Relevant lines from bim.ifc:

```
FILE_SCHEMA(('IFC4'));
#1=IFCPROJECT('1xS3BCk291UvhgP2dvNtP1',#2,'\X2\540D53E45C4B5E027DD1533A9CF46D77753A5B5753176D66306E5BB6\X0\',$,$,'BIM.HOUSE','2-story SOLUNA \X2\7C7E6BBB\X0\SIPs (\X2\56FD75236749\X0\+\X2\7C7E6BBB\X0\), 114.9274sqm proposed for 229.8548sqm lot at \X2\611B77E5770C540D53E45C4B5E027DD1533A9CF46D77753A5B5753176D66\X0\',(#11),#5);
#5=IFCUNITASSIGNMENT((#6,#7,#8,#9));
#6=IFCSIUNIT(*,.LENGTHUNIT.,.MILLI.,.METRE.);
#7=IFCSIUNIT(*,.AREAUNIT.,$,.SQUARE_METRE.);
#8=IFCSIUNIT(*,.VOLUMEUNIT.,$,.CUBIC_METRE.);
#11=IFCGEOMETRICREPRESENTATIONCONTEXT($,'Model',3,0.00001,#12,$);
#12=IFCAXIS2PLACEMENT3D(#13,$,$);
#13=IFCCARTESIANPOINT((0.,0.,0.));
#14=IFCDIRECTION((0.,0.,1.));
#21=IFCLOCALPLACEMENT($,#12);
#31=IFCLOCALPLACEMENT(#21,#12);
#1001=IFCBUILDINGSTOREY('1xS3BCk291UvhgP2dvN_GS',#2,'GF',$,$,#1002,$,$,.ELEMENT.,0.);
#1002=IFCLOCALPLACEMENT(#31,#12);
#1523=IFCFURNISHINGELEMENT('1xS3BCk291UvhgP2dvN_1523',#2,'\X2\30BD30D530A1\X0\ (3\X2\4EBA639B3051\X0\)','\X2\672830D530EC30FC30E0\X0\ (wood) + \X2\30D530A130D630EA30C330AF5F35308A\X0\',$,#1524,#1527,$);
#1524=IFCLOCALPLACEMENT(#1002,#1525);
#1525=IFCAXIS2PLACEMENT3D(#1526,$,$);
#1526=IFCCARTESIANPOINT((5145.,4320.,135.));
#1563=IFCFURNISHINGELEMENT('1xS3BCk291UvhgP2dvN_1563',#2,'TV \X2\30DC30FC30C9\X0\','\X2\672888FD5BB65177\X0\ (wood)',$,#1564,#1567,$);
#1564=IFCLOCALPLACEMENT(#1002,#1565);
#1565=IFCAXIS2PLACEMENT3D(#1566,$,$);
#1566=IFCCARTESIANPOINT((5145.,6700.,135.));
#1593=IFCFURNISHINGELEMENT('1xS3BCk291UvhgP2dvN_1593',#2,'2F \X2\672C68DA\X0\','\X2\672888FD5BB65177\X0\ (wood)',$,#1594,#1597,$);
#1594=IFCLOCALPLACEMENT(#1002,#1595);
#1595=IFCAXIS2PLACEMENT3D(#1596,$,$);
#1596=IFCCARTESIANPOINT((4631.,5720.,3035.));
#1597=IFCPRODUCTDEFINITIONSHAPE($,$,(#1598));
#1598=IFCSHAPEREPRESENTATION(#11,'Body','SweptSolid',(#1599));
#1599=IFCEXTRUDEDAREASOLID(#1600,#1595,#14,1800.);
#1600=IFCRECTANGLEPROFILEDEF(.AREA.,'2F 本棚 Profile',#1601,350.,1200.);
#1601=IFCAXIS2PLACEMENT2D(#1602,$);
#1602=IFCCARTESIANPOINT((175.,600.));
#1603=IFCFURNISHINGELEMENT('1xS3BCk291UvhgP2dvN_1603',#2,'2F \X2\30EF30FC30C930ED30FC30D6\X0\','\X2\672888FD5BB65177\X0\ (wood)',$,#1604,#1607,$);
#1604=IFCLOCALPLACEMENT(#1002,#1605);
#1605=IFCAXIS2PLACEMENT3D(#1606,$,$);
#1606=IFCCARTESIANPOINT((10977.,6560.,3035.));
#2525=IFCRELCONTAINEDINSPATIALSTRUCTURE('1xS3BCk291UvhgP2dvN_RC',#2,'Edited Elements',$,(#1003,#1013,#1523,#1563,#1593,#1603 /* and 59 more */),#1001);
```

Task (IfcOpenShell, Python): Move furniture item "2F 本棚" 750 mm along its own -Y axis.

```python
import ifcopenshell
import ifcopenshell.api.geometry
import ifcopenshell.util.placement
import ifcopenshell.util.unit

model = ifcopenshell.open("bim.ifc")
unit_scale = ifcopenshell.util.unit.calculate_unit_scale(model)

item = model.by_id(1593)
matrix = ifcopenshell.util.placement.get_local_placement(item.ObjectPlacement)
matrix[:3, 3] -= matrix[:3, 1] * 0.75 / unit_scale
ifcopenshell.api.geometry.edit_object_placement(model, product=item, matrix=matrix, is_si=False)

print(ifcopenshell.util.placement.get_local_placement(item.ObjectPlacement).round(3) + 0.0)

model.write("bim_updated.ifc")
```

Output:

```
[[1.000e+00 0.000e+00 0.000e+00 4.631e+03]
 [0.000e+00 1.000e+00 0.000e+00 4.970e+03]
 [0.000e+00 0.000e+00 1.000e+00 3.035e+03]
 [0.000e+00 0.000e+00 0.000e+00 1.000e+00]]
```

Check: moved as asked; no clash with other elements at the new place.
